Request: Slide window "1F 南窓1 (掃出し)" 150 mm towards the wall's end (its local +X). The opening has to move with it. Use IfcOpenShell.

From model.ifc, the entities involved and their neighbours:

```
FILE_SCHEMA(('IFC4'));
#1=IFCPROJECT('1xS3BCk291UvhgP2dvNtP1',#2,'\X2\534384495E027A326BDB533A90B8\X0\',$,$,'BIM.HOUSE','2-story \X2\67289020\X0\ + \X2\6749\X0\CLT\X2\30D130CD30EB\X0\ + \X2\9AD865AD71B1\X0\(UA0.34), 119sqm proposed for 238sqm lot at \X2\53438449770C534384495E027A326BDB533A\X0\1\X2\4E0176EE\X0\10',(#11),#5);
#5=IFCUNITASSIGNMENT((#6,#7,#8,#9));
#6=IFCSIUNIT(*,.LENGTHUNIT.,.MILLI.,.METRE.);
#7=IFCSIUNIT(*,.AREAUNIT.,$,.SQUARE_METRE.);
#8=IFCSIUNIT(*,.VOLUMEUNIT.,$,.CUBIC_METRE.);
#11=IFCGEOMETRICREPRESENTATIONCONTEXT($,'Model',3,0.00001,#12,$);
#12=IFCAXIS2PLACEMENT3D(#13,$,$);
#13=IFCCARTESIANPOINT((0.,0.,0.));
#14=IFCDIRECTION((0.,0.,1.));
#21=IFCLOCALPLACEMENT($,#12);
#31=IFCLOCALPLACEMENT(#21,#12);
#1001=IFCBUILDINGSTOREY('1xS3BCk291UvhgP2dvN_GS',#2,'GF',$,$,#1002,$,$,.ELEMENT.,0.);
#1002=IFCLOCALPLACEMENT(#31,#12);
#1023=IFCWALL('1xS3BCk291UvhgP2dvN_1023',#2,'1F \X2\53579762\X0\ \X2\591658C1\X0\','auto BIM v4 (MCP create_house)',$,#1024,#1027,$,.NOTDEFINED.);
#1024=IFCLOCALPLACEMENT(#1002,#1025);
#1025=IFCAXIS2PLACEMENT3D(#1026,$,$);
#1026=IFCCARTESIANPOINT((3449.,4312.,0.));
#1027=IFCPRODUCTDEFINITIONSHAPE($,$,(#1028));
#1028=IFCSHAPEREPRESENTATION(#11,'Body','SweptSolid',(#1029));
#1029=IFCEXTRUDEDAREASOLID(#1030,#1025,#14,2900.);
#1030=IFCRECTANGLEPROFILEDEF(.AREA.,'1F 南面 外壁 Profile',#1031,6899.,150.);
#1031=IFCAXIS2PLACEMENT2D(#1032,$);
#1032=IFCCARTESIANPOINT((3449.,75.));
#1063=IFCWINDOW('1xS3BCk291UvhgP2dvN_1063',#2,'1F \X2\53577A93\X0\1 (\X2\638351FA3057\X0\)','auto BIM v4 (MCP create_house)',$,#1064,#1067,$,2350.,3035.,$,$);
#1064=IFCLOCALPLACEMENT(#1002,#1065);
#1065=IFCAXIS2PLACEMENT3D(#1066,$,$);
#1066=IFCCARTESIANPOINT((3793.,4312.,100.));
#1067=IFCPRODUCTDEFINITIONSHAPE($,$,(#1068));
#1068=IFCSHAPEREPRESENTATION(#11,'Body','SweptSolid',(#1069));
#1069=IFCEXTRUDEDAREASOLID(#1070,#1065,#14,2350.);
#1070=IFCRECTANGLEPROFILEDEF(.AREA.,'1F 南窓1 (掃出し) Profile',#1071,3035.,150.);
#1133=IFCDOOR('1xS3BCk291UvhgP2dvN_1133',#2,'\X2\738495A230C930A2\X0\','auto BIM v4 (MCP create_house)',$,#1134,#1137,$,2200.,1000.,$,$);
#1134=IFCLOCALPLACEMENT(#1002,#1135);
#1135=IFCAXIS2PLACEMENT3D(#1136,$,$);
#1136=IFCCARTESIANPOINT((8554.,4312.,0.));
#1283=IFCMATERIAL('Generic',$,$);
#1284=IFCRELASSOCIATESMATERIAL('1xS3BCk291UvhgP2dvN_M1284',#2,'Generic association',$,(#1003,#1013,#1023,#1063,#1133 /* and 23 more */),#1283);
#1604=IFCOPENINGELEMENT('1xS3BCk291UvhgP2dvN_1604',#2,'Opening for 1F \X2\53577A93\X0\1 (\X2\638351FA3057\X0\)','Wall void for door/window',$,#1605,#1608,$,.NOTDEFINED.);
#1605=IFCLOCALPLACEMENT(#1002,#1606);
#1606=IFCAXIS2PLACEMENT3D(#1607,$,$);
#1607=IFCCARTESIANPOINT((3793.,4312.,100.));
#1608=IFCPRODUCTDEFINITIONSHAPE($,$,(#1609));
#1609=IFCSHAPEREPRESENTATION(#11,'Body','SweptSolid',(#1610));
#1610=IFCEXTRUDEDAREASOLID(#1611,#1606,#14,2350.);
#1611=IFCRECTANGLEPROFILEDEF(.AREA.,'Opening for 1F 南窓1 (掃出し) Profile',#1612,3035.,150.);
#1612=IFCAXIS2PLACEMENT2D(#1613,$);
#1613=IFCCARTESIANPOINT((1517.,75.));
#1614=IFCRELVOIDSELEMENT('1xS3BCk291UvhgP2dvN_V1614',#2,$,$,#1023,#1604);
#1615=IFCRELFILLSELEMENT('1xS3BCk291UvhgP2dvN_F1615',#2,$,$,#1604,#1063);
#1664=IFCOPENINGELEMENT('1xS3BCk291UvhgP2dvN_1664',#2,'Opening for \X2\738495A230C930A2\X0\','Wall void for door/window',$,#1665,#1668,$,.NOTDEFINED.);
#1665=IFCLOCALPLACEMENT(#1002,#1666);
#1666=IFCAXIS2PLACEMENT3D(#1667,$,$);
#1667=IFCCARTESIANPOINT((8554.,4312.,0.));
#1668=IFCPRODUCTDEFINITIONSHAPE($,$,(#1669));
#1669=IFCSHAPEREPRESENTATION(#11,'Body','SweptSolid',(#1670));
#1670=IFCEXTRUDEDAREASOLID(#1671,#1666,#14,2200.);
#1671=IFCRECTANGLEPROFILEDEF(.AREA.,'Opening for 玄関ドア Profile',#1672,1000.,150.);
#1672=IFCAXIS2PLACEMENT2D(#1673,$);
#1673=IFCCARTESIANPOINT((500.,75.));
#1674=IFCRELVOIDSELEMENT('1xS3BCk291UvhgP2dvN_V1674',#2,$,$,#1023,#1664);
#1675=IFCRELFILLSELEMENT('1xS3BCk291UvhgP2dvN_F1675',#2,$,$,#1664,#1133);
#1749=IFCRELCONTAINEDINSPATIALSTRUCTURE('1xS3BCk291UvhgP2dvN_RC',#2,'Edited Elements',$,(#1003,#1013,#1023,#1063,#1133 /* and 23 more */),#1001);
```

```python
import ifcopenshell
import ifcopenshell.api.geometry
import ifcopenshell.util.placement
import ifcopenshell.util.unit

model = ifcopenshell.open("model.ifc")
unit_scale = ifcopenshell.util.unit.calculate_unit_scale(model)

window = model.by_guid("1xS3BCk291UvhgP2dvN_1063")
opening = window.FillsVoids[0].RelatingOpeningElement
wall = opening.VoidsElements[0].RelatingBuildingElement

wall_matrix = ifcopenshell.util.placement.get_local_placement(wall.ObjectPlacement)
shift = wall_matrix[:3, 0] * 0.15 / unit_scale
before = ifcopenshell.util.placement.get_local_placement(window.ObjectPlacement)[:3, 3].copy()

# The window is not placed relative to its opening, so move both.
for product in (opening, window):
    matrix = ifcopenshell.util.placement.get_local_placement(product.ObjectPlacement)
    matrix[:3, 3] += shift
    ifcopenshell.api.geometry.edit_object_placement(model, product=product, matrix=matrix, is_si=False)

after = ifcopenshell.util.placement.get_local_placement(window.ObjectPlacement)[:3, 3]
print("window moved by", (after - before).round(3) + 0.0)

model.write("model_updated.ifc")
```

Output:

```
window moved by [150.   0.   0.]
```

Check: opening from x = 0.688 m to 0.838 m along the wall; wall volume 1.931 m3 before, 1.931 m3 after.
